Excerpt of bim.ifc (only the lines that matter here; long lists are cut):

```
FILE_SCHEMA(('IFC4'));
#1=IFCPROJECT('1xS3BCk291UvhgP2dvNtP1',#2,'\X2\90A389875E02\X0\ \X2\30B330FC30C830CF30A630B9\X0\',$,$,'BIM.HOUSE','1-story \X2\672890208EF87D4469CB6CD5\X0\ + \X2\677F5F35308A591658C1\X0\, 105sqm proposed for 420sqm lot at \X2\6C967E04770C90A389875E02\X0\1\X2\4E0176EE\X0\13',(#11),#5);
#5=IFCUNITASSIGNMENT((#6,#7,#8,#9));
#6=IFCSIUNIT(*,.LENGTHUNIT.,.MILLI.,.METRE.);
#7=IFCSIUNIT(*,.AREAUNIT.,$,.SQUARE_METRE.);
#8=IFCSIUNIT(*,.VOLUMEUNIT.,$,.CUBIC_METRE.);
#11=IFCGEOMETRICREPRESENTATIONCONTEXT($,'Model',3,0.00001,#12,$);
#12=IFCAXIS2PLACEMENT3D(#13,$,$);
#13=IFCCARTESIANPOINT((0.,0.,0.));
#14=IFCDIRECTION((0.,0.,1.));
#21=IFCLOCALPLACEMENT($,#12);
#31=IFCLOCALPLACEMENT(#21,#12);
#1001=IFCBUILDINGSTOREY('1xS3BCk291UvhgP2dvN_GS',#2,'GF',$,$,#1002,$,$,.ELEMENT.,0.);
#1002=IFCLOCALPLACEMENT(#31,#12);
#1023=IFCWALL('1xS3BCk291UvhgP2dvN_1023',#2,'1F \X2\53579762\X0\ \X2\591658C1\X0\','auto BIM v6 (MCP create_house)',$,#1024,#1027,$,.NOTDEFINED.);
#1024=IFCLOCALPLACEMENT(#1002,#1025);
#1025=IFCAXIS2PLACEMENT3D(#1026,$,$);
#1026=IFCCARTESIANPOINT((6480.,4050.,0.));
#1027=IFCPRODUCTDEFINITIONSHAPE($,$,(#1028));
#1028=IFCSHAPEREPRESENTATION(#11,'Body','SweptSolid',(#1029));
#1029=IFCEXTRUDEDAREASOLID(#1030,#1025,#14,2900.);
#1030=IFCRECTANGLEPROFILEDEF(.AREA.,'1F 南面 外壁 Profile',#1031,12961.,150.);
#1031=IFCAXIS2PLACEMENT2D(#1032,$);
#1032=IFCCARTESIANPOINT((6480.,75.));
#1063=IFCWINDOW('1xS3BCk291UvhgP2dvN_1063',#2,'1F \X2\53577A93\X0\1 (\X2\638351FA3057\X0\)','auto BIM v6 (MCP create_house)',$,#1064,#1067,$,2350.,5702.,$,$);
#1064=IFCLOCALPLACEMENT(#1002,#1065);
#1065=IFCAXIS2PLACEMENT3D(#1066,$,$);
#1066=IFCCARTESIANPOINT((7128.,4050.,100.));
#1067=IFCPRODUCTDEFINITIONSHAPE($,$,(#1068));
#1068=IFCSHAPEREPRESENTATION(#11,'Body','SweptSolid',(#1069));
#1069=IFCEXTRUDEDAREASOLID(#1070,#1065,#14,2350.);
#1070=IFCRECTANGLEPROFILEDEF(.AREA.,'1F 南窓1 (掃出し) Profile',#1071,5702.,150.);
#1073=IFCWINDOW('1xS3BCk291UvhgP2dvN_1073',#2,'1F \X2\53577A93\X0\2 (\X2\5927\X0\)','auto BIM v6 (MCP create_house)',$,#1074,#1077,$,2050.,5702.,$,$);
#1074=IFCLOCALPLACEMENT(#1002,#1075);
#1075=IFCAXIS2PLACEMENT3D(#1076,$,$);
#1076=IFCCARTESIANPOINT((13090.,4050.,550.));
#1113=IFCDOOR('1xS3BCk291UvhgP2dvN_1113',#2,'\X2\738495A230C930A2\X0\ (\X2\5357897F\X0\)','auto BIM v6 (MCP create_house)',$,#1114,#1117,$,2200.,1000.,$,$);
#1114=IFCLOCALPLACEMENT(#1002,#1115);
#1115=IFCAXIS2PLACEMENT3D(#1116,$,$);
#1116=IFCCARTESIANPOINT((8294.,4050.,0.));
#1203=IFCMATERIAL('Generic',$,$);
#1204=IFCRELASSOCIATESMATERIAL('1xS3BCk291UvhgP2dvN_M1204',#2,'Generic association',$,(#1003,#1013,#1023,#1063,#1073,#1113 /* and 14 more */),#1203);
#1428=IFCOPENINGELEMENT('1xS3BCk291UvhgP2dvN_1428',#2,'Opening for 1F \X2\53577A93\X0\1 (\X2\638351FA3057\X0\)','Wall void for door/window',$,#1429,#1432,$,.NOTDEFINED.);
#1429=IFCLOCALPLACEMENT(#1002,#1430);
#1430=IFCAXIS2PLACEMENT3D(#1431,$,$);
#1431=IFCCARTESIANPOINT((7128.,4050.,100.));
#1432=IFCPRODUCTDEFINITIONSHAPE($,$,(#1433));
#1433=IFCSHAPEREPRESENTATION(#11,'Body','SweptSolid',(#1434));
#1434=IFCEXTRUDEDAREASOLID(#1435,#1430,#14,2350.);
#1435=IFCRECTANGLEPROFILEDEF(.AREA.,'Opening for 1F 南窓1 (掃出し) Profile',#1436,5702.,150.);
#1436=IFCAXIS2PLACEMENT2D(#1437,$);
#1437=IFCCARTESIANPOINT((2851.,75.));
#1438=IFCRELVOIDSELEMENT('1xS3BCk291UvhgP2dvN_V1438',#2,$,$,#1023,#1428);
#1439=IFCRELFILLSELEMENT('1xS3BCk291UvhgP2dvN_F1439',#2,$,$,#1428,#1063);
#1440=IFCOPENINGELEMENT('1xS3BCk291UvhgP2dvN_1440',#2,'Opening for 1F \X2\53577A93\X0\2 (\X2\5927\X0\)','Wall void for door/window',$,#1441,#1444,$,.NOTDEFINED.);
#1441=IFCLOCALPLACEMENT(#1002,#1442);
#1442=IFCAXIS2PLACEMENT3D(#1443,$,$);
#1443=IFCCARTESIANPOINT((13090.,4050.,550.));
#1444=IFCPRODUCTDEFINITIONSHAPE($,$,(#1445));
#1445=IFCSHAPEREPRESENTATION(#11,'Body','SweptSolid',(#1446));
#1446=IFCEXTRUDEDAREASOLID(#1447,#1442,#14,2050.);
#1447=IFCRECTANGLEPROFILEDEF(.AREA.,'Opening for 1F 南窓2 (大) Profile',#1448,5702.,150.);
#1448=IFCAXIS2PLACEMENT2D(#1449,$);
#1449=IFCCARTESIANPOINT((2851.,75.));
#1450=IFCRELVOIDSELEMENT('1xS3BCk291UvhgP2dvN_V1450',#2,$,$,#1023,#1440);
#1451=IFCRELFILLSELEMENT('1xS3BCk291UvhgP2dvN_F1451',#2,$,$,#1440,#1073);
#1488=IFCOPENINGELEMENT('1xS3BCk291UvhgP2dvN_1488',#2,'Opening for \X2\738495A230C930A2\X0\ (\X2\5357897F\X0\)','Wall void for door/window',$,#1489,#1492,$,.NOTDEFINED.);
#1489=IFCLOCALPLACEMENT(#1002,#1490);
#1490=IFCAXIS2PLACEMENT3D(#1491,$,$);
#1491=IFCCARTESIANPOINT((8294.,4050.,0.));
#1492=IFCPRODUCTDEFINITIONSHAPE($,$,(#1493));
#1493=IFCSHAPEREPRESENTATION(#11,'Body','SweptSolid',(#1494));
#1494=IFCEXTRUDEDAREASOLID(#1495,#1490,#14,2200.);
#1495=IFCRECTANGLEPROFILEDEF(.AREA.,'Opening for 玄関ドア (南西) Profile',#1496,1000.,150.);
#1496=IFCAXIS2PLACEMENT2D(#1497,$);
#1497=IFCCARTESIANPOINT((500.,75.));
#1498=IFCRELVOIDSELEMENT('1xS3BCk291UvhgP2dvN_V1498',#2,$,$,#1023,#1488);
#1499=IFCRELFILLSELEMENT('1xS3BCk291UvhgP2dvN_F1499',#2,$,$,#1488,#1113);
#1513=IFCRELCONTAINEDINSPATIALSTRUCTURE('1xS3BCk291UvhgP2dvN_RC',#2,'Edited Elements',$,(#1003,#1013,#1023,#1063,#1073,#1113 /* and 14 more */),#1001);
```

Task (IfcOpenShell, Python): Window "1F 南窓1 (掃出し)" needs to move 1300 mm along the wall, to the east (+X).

```python
import ifcopenshell
import ifcopenshell.api.geometry
import ifcopenshell.util.placement

model = ifcopenshell.open("bim.ifc")

window = model.by_guid("1xS3BCk291UvhgP2dvN_1063")
opening = window.FillsVoids[0].RelatingOpeningElement
wall = opening.VoidsElements[0].RelatingBuildingElement

wall_matrix = ifcopenshell.util.placement.get_local_placement(wall.ObjectPlacement)
shift = wall_matrix[:3, 0] * 1300.0
before = ifcopenshell.util.placement.get_local_placement(window.ObjectPlacement)[:3, 3].copy()

# The window is not placed relative to its opening, so move both.
for product in (opening, window):
    matrix = ifcopenshell.util.placement.get_local_placement(product.ObjectPlacement)
    matrix[:3, 3] += shift
    ifcopenshell.api.geometry.edit_object_placement(model, product=product, matrix=matrix, is_si=False)

after = ifcopenshell.util.placement.get_local_placement(window.ObjectPlacement)[:3, 3]
print("window moved by", (after - before).round(3) + 0.0)

model.write("bim_rev.ifc")
```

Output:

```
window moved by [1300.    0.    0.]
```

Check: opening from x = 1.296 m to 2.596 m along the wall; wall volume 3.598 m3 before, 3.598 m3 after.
